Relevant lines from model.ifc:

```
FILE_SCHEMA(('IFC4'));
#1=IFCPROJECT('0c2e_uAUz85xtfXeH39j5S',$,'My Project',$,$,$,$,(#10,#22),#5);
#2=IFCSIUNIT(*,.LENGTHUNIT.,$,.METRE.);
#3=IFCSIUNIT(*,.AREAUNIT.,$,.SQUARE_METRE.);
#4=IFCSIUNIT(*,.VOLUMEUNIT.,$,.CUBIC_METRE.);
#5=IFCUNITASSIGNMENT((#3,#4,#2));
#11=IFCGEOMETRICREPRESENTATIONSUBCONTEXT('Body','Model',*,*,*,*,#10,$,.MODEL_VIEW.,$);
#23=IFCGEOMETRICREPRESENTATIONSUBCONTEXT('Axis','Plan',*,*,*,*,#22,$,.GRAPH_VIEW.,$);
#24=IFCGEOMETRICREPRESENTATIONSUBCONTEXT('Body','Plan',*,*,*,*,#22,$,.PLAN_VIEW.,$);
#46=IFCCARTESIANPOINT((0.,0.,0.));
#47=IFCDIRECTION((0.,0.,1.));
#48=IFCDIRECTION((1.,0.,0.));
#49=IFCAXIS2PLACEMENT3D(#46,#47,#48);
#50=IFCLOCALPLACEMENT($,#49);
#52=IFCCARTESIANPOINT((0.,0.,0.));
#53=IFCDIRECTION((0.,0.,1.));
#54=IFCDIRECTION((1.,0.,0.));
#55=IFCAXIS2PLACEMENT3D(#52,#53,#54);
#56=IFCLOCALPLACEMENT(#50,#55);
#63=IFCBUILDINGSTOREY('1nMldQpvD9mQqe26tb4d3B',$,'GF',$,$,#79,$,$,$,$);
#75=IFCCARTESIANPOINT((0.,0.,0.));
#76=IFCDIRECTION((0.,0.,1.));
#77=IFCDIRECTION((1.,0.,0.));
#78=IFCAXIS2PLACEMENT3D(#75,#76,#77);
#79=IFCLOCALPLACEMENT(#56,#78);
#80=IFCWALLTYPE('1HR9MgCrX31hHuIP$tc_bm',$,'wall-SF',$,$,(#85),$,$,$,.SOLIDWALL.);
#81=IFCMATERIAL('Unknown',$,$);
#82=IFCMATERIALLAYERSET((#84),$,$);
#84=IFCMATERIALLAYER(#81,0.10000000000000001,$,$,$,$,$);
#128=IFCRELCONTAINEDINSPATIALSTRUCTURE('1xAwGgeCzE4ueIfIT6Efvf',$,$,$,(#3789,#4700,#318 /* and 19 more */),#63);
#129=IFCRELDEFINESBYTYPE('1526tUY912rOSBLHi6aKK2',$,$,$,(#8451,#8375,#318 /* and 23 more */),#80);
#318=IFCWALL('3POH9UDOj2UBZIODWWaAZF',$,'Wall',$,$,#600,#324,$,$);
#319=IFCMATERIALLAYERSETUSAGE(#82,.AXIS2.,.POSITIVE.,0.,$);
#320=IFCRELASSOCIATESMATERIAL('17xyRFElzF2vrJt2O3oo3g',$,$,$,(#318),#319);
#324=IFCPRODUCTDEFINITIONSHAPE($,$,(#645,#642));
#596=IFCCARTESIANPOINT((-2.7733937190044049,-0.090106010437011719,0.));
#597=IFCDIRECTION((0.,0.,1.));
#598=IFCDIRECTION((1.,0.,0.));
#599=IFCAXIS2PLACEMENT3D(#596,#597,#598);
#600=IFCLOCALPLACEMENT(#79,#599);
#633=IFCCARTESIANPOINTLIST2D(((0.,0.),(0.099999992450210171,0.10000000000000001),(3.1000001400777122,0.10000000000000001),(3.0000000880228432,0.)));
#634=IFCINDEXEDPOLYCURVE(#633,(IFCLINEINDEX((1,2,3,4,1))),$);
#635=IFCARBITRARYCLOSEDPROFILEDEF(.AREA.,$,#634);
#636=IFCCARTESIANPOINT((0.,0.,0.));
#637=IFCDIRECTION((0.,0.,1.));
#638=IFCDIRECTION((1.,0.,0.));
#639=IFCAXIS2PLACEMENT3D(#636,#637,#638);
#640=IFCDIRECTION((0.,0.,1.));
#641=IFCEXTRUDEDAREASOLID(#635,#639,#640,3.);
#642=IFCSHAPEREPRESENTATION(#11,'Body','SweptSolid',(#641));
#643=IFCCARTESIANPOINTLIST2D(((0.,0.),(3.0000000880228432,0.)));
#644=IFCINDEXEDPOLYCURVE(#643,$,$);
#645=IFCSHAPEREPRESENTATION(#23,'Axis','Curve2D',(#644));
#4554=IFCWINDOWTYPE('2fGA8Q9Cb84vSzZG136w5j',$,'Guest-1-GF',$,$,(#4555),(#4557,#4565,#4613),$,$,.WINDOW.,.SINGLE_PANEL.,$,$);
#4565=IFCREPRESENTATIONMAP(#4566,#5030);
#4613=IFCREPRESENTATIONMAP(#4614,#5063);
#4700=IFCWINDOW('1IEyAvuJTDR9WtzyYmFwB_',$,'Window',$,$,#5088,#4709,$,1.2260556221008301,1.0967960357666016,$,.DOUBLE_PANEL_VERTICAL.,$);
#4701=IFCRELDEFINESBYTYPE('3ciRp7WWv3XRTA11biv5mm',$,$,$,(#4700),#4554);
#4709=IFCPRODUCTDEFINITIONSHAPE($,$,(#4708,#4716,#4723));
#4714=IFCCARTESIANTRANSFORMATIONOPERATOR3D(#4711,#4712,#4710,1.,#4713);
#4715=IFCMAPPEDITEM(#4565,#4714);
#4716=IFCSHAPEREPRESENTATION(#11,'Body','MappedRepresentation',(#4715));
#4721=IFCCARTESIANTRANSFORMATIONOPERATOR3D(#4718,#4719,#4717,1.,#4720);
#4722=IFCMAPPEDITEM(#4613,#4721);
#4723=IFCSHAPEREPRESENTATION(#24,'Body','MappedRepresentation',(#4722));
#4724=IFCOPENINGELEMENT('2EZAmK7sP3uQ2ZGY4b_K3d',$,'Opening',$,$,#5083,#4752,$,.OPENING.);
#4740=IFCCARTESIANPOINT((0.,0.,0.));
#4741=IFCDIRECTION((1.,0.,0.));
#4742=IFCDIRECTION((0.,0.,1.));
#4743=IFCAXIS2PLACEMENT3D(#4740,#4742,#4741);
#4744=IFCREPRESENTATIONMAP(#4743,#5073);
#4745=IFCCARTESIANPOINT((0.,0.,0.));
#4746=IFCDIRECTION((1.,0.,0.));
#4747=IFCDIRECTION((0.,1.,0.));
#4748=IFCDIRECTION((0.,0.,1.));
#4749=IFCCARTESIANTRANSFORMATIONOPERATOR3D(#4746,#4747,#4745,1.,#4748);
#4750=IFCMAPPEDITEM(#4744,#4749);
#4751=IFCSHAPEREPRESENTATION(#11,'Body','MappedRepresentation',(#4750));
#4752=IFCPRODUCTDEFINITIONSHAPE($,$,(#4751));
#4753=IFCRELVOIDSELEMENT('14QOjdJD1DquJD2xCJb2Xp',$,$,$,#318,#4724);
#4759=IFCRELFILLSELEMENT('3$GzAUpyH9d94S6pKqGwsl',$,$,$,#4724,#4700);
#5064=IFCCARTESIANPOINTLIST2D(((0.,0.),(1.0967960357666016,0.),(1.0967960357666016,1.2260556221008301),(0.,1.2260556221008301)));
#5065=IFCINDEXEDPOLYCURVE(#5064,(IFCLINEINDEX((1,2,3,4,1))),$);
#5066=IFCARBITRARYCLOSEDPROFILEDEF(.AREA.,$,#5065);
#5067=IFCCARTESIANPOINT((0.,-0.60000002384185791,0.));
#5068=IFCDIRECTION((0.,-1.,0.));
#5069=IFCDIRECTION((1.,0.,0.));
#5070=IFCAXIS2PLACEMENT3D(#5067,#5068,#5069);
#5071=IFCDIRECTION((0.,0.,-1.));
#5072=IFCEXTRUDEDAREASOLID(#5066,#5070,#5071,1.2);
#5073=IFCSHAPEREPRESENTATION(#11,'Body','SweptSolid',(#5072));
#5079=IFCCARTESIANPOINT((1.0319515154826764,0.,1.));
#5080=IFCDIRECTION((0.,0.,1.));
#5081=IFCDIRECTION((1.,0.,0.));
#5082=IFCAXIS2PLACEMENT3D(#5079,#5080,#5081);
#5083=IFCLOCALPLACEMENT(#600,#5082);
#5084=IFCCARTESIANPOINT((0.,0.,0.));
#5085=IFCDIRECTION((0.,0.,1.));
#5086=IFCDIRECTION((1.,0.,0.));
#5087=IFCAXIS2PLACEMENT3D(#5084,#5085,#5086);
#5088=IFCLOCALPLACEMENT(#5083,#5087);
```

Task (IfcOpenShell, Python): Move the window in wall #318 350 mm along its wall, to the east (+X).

```python
import ifcopenshell
import ifcopenshell.api.geometry
import ifcopenshell.util.placement
import ifcopenshell.util.unit

model = ifcopenshell.open("model.ifc")
unit_scale = ifcopenshell.util.unit.calculate_unit_scale(model)

window = model.by_id(4700)
opening = window.FillsVoids[0].RelatingOpeningElement
wall = opening.VoidsElements[0].RelatingBuildingElement

wall_matrix = ifcopenshell.util.placement.get_local_placement(wall.ObjectPlacement)
shift = wall_matrix[:3, 0] * 0.35 / unit_scale
before = ifcopenshell.util.placement.get_local_placement(window.ObjectPlacement)[:3, 3].copy()

# The window is placed relative to its opening, so it follows when the opening moves.
matrix = ifcopenshell.util.placement.get_local_placement(opening.ObjectPlacement)
matrix[:3, 3] += shift
ifcopenshell.api.geometry.edit_object_placement(
    model, product=opening, matrix=matrix, is_si=False, should_transform_children=True
)

after = ifcopenshell.util.placement.get_local_placement(window.ObjectPlacement)[:3, 3]
print("window moved by", (after - before).round(3) + 0.0)

model.write("model_v2.ifc")
```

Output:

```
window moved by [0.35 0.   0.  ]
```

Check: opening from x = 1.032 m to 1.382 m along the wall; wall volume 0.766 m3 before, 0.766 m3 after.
